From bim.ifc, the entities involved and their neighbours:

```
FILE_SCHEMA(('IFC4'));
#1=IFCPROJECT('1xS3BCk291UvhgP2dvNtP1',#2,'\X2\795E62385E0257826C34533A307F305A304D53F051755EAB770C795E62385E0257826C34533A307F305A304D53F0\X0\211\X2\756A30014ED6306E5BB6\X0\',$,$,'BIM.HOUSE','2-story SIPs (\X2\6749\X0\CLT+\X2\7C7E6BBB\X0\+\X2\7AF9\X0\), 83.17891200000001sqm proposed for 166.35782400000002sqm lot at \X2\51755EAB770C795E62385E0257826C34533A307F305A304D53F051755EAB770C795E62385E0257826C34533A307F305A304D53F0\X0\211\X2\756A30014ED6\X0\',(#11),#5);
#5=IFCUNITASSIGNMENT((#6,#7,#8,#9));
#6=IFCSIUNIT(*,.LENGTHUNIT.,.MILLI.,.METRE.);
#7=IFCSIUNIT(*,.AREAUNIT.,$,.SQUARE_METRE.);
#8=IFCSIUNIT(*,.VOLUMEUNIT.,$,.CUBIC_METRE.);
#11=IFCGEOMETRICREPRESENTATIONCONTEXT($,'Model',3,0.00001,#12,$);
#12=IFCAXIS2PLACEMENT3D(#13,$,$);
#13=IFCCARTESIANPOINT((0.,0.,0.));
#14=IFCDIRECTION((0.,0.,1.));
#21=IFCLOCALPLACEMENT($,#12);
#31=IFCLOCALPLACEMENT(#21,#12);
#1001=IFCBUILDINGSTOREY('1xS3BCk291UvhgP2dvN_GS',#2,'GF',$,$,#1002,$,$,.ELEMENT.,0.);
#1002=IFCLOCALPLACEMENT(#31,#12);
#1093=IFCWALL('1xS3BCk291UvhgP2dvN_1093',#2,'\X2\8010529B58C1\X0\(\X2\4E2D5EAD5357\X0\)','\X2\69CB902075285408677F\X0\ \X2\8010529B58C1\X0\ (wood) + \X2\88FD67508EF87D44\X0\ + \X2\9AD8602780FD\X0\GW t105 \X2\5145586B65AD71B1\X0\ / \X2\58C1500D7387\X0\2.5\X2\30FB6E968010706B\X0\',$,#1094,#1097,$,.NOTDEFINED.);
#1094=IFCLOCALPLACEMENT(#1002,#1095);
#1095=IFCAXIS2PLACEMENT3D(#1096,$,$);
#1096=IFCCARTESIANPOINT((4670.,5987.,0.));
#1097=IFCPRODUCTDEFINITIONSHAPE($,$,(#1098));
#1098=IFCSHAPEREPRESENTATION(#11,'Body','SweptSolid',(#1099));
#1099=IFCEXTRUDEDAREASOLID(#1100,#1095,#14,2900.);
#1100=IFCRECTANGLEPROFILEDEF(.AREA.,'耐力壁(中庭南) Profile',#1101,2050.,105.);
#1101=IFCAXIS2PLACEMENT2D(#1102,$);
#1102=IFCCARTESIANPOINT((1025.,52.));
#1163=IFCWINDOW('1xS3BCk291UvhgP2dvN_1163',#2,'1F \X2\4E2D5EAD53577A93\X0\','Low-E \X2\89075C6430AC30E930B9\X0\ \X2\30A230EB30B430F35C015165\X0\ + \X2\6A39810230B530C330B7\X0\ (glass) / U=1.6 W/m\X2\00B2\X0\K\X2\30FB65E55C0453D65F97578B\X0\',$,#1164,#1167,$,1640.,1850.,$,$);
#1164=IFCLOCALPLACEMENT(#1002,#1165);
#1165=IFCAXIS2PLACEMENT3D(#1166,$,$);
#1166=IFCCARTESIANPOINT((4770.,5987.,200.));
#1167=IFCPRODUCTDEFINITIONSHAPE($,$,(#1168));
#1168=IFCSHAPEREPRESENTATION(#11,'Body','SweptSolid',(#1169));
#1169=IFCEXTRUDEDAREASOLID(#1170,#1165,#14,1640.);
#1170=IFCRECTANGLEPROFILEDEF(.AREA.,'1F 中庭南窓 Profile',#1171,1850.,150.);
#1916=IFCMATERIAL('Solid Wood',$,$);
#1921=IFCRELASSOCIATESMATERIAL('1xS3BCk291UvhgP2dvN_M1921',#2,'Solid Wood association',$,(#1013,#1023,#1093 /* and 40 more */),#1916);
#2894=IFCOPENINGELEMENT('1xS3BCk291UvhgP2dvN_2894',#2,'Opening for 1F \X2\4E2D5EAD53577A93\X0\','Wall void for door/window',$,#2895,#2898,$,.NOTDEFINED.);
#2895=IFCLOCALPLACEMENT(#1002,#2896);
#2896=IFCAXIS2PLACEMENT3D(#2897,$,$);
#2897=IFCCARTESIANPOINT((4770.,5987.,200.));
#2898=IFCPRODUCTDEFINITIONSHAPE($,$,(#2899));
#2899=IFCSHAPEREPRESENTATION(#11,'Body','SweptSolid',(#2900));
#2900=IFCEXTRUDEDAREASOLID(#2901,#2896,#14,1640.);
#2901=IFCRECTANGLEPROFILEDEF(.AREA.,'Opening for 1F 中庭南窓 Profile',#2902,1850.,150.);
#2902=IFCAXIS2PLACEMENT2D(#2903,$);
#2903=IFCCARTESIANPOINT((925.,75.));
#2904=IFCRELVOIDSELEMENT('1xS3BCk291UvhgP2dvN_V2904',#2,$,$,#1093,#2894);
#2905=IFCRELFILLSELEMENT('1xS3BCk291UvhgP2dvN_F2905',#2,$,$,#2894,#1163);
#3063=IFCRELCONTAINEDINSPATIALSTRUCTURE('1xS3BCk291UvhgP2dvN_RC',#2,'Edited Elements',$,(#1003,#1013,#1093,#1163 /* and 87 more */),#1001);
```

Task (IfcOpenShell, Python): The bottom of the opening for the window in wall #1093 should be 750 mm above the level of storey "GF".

```python
import numpy as np
import ifcopenshell
import ifcopenshell.api.geometry
import ifcopenshell.geom
import ifcopenshell.util.element
import ifcopenshell.util.placement
import ifcopenshell.util.shape
import ifcopenshell.util.unit

model = ifcopenshell.open("bim.ifc")
unit_scale = ifcopenshell.util.unit.calculate_unit_scale(model)

window = model.by_guid("1xS3BCk291UvhgP2dvN_1163")
opening = window.FillsVoids[0].RelatingOpeningElement
storey = ifcopenshell.util.element.get_container(window, ifc_class="IfcBuildingStorey")
level = ifcopenshell.util.placement.get_local_placement(storey.ObjectPlacement)[2, 3]

# The opening's origin need not be at the sill, so measure its lowest point.
shape = ifcopenshell.geom.create_shape(ifcopenshell.geom.settings(), opening)
bottom = ifcopenshell.util.shape.get_shape_bottom_elevation(shape, shape.geometry) / unit_scale
dz = level + 0.75 / unit_scale - bottom

shift = np.array([0.0, 0.0, dz])
# The window is not placed relative to its opening, so move both.
for product in (opening, window):
    matrix = ifcopenshell.util.placement.get_local_placement(product.ObjectPlacement)
    matrix[:3, 3] += shift
    ifcopenshell.api.geometry.edit_object_placement(model, product=product, matrix=matrix, is_si=False)

print(f"moved by {dz * unit_scale:+.3f} m")

model.write("bim_v2.ifc")
```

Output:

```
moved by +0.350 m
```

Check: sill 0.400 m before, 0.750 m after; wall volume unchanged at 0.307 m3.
